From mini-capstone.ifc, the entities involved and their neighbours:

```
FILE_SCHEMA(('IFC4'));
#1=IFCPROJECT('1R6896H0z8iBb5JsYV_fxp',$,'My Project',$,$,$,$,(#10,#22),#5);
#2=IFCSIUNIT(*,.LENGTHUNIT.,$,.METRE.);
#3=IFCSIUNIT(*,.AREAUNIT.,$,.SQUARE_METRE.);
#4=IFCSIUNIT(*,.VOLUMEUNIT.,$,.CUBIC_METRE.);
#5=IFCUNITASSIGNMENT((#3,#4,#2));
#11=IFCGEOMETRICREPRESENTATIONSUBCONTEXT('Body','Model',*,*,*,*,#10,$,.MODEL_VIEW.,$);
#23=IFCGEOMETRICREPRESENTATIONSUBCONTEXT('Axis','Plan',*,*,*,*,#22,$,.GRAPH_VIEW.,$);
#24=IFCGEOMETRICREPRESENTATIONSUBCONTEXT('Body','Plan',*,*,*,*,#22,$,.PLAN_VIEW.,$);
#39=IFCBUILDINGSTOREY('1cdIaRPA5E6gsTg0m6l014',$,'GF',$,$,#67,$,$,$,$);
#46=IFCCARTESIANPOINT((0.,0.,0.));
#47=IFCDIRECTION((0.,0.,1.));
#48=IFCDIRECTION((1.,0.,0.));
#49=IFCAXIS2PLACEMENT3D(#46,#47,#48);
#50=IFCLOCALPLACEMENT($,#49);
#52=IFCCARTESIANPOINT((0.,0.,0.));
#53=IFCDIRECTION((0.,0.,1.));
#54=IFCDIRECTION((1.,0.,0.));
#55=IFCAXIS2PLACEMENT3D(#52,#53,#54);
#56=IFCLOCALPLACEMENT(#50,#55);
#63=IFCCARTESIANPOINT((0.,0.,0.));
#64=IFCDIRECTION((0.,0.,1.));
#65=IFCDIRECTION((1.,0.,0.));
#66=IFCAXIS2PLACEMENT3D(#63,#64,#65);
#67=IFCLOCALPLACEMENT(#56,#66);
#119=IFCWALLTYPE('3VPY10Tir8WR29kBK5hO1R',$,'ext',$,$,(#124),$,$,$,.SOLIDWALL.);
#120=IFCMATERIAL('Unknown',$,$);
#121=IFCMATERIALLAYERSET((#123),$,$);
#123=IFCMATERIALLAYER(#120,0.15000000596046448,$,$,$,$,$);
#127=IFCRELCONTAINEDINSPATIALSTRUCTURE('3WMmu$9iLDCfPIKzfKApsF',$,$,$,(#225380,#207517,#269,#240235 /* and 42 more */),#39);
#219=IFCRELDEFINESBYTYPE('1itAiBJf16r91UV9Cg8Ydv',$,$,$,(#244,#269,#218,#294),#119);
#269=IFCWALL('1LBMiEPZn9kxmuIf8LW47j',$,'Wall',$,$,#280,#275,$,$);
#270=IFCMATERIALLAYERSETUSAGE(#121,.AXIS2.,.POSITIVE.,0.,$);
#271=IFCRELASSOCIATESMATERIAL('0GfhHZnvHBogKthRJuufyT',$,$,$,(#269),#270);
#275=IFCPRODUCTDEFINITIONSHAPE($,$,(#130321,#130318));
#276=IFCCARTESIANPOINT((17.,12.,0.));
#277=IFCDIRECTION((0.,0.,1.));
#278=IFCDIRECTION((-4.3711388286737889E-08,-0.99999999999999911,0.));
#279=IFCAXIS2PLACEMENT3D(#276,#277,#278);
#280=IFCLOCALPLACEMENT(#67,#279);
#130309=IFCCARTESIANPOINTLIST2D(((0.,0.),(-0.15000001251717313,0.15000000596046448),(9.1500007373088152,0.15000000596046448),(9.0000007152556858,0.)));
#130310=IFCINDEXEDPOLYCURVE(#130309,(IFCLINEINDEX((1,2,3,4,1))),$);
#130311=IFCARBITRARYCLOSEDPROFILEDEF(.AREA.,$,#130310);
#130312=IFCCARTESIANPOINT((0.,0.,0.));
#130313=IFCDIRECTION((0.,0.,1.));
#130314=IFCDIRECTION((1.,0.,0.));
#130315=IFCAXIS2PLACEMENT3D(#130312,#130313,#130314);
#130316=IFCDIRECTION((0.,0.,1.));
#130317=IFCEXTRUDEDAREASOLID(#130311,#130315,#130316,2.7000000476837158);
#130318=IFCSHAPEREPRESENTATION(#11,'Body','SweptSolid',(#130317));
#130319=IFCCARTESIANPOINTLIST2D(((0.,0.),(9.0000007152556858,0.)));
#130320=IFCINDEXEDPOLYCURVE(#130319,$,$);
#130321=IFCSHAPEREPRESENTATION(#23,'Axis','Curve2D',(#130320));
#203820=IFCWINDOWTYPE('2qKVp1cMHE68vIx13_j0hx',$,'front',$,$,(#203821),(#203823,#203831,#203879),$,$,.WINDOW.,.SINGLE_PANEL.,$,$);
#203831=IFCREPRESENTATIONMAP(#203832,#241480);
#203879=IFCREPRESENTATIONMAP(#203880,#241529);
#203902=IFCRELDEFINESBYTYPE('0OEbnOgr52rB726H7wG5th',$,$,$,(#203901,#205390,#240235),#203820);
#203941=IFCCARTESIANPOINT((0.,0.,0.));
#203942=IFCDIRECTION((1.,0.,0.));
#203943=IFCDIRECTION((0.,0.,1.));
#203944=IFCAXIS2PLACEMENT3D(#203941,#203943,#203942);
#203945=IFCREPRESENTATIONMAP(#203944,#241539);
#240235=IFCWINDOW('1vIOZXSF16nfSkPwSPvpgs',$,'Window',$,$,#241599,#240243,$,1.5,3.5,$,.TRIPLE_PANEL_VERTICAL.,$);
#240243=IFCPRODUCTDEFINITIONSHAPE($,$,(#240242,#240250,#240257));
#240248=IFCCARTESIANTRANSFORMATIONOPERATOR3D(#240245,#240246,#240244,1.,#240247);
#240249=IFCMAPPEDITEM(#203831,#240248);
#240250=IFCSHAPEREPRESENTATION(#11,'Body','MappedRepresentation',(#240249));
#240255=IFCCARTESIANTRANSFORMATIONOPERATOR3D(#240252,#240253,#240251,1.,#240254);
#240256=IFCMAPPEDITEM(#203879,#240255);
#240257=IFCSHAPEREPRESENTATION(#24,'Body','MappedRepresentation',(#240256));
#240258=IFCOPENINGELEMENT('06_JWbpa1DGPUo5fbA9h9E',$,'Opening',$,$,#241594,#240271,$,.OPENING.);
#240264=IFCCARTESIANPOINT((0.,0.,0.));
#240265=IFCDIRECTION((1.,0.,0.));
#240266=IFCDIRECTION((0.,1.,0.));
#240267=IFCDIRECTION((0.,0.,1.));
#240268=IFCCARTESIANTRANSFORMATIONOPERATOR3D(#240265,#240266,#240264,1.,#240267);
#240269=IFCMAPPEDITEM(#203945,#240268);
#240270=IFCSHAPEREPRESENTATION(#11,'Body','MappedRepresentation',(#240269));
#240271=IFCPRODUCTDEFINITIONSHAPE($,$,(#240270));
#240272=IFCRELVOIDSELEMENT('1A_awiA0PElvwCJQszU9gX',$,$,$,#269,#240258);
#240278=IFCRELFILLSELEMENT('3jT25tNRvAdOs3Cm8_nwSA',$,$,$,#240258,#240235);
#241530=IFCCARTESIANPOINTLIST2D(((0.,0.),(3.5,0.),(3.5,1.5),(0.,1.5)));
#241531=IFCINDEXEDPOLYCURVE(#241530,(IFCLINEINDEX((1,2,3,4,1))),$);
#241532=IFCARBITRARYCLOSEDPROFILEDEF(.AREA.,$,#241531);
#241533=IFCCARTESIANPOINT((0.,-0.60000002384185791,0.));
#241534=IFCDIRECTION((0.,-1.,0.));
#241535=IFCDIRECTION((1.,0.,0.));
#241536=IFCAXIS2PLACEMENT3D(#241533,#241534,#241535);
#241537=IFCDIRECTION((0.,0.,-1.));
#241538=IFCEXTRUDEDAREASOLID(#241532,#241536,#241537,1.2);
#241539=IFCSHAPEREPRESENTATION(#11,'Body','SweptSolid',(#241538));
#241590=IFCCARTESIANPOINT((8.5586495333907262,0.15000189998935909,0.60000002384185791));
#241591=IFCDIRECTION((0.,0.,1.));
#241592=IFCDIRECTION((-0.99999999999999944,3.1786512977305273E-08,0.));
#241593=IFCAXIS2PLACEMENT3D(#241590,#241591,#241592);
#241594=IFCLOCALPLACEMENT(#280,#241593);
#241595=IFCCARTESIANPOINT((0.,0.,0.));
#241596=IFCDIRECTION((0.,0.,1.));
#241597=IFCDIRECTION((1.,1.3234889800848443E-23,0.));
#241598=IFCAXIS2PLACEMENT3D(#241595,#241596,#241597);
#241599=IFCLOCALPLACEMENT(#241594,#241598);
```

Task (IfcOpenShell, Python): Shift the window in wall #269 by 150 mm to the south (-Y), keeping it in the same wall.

```python
import ifcopenshell
import ifcopenshell.api.geometry
import ifcopenshell.util.placement
import ifcopenshell.util.unit

model = ifcopenshell.open("mini-capstone.ifc")
unit_scale = ifcopenshell.util.unit.calculate_unit_scale(model)

window = model.by_guid("1vIOZXSF16nfSkPwSPvpgs")
opening = window.FillsVoids[0].RelatingOpeningElement
wall = opening.VoidsElements[0].RelatingBuildingElement

wall_matrix = ifcopenshell.util.placement.get_local_placement(wall.ObjectPlacement)
shift = wall_matrix[:3, 0] * 0.15 / unit_scale
before = ifcopenshell.util.placement.get_local_placement(window.ObjectPlacement)[:3, 3].copy()

# The window is placed relative to its opening, so it follows when the opening moves.
matrix = ifcopenshell.util.placement.get_local_placement(opening.ObjectPlacement)
matrix[:3, 3] += shift
ifcopenshell.api.geometry.edit_object_placement(
    model, product=opening, matrix=matrix, is_si=False, should_transform_children=True
)

after = ifcopenshell.util.placement.get_local_placement(window.ObjectPlacement)[:3, 3]
print("window moved by", (after - before).round(3) + 0.0)

model.write("mini-capstone_edited.ifc")
```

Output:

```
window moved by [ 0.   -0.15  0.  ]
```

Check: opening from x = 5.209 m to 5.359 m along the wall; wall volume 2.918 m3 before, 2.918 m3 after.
